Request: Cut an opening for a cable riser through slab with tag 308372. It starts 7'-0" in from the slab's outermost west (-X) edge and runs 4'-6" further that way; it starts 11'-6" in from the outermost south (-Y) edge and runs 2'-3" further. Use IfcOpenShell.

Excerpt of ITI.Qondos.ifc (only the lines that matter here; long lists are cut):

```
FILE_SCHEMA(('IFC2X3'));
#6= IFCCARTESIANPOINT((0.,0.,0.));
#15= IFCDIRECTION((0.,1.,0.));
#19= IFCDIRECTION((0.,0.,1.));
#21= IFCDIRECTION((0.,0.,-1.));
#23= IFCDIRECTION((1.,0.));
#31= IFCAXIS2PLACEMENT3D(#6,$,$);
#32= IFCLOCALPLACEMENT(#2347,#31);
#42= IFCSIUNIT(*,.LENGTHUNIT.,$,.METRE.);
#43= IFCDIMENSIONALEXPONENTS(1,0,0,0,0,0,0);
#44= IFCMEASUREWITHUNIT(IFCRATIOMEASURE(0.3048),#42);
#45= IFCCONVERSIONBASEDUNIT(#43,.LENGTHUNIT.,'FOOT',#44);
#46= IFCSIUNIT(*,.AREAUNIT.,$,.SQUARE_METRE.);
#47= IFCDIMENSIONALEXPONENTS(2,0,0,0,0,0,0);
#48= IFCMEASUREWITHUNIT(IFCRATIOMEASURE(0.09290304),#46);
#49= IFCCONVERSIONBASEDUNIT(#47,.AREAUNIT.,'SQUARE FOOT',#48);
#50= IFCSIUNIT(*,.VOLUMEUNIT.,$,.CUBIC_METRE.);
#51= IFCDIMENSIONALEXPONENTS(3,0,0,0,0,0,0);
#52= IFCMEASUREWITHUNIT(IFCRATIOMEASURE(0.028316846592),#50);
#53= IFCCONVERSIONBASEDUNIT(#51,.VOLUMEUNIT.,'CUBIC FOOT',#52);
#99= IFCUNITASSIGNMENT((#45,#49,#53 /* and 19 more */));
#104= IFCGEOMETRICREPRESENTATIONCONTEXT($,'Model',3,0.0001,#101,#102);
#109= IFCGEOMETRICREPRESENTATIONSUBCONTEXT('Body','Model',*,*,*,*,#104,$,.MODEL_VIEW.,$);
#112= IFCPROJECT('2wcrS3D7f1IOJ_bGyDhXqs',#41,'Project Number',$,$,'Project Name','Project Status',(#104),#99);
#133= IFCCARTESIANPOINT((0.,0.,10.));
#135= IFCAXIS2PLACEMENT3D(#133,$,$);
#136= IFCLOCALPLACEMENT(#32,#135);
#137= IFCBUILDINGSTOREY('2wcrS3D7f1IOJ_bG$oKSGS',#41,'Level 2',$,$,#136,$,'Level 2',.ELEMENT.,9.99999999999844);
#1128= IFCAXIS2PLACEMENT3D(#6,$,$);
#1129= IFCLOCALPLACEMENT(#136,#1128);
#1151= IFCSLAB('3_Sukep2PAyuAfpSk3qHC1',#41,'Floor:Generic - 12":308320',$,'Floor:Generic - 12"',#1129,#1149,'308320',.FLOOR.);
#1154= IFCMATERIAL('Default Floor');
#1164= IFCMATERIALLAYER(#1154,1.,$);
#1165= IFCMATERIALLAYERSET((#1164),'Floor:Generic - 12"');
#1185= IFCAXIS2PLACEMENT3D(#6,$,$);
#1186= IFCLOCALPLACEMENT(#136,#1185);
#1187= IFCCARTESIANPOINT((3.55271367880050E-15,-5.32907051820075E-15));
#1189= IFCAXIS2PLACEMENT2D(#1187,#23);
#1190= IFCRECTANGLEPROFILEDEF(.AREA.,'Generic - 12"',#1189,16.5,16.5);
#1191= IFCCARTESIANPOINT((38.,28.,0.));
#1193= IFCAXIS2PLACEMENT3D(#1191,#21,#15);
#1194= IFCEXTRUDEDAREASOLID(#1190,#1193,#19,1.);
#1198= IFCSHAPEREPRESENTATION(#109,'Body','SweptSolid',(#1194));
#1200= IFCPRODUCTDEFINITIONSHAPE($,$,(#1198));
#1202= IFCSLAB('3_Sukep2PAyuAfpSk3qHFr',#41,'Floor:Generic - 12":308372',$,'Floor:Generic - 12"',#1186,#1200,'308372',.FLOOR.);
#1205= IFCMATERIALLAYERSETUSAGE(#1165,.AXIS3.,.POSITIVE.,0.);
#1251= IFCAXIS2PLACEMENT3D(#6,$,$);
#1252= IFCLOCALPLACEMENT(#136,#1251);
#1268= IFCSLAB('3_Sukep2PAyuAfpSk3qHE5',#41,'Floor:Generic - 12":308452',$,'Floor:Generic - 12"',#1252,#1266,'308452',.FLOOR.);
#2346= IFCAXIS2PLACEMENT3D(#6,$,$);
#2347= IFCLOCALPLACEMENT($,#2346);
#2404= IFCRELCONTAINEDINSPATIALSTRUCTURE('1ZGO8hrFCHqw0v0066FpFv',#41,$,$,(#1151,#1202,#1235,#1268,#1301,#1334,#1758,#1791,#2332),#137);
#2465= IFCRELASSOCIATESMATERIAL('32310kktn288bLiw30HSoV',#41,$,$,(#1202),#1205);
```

```python
import numpy as np
import ifcopenshell
import ifcopenshell.api.feature
import ifcopenshell.api.geometry
import ifcopenshell.api.root
import ifcopenshell.geom
import ifcopenshell.util.placement
import ifcopenshell.util.representation
import ifcopenshell.util.shape
import ifcopenshell.util.unit

model = ifcopenshell.open("ITI.Qondos.ifc")
unit_scale = ifcopenshell.util.unit.calculate_unit_scale(model)
settings = ifcopenshell.geom.settings()


def volume(element):
    """Net volume in cubic metres, openings subtracted."""
    shape = ifcopenshell.geom.create_shape(settings, element)
    return ifcopenshell.util.shape.get_volume(shape.geometry)


slab = model.by_guid("3_Sukep2PAyuAfpSk3qHFr")
before = volume(slab)

# Extent in the slab's own axes, in metres. The edges named are its -X and -Y sides.
slab_shape = ifcopenshell.geom.create_shape(settings, slab)
vertices = ifcopenshell.util.shape.get_vertices(slab_shape.geometry)
x_min, y_min, bottom = vertices.min(axis=0)
top = vertices[:, 2].max()

opening = ifcopenshell.api.root.create_entity(model, ifc_class="IfcOpeningElement", name="Cable riser opening")
context = ifcopenshell.util.representation.get_context(model, "Model", "Body", "MODEL_VIEW")
width, depth = 1.3716, 0.6858
outline = [(0.0, 0.0), (width, 0.0), (width, depth), (0.0, depth), (0.0, 0.0)]
# Overshoot both faces by 50 mm so the cut is clean.
shape = ifcopenshell.api.geometry.add_slab_representation(
    model, context=context, depth=top - bottom + 0.1, polyline=outline
)
ifcopenshell.api.geometry.assign_representation(model, product=opening, representation=shape)

matrix = ifcopenshell.util.placement.get_local_placement(slab.ObjectPlacement)
matrix[:, 3] = matrix @ np.append(np.array([x_min + 2.1336, y_min + 3.5052, bottom - 0.05]) / unit_scale, 1.0)
ifcopenshell.api.geometry.edit_object_placement(model, product=opening, matrix=matrix, is_si=False)
ifcopenshell.api.feature.add_feature(model, feature=opening, element=slab)

after = volume(slab)

print(f"slab volume {before:.3f} -> {after:.3f} m3")

model.write("ITI.Qondos-out.ifc")
```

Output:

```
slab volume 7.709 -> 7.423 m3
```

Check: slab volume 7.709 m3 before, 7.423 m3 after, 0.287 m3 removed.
